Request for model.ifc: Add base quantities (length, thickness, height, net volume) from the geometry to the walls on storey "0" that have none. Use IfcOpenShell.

First a look at what the model holds.

```python
import ifcopenshell
import ifcopenshell.util.element
import ifcopenshell.util.unit

model = ifcopenshell.open("model.ifc")
print(model.schema)
for unit_type in ("LENGTHUNIT", "AREAUNIT", "VOLUMEUNIT"):
    print(unit_type, ifcopenshell.util.unit.calculate_unit_scale(model, unit_type))
storey = next(s for s in model.by_type("IfcBuildingStorey") if s.Name == "0")
walls = [e for e in ifcopenshell.util.element.get_decomposition(storey) if e.is_a("IfcWall")]
for e in sorted(walls, key=lambda e: e.id()):
    print(e.id(), e.is_a(), e.Name, list(ifcopenshell.util.element.get_psets(e, qtos_only=True)), sep=" | ")
```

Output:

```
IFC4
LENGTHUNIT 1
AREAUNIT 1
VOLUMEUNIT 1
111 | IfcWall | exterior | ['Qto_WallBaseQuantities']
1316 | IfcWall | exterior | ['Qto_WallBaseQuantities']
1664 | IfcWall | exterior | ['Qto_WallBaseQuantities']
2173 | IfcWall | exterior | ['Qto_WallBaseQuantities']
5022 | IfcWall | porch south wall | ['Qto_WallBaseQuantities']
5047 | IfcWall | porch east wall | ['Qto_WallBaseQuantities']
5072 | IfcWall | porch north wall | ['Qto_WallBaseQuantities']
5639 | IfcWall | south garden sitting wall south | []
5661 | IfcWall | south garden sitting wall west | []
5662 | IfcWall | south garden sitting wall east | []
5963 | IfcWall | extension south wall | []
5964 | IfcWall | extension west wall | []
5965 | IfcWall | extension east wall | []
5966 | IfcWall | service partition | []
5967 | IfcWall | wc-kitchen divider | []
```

```python
import ifcopenshell
import ifcopenshell.api.pset
import ifcopenshell.geom
import ifcopenshell.util.element
import ifcopenshell.util.shape
import ifcopenshell.util.unit

model = ifcopenshell.open("model.ifc")
unit_scale = ifcopenshell.util.unit.calculate_unit_scale(model)
volume_scale = ifcopenshell.util.unit.calculate_unit_scale(model, "VOLUMEUNIT")
settings = ifcopenshell.geom.settings()

storey = next(s for s in model.by_type("IfcBuildingStorey") if s.Name == "0")
walls = [e for e in ifcopenshell.util.element.get_decomposition(storey) if e.is_a("IfcWall")]

for e in sorted(walls, key=lambda e: e.id()):
    if ifcopenshell.util.element.get_psets(e, qtos_only=True, should_inherit=False):
        continue
    # Geometry comes back in metres, in the element's own axes.
    shape = ifcopenshell.geom.create_shape(settings, e)
    values = {
        "Length": ifcopenshell.util.shape.get_x(shape.geometry) / unit_scale,
        "Width": ifcopenshell.util.shape.get_y(shape.geometry) / unit_scale,
        "Height": ifcopenshell.util.shape.get_z(shape.geometry) / unit_scale,
        "NetVolume": ifcopenshell.util.shape.get_volume(shape.geometry) / volume_scale,
    }
    qto = ifcopenshell.api.pset.add_qto(model, product=e, name="Qto_WallBaseQuantities")
    ifcopenshell.api.pset.edit_qto(model, qto=qto, properties=values)
    print(e.id(), {k: round(v, 3) for k, v in values.items()})

model.write("model_v2.ifc")
```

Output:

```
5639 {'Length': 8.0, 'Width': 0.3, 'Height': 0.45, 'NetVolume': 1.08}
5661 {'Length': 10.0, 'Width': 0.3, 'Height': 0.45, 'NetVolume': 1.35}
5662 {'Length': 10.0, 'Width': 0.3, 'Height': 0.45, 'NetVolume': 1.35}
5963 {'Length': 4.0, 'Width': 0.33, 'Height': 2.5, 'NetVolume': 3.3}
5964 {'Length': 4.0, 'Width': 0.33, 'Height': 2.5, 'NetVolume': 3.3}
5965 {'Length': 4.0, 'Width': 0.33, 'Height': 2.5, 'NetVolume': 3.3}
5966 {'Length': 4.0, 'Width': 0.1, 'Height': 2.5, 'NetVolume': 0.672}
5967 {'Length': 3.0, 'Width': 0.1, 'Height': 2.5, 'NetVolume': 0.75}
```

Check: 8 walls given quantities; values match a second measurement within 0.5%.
